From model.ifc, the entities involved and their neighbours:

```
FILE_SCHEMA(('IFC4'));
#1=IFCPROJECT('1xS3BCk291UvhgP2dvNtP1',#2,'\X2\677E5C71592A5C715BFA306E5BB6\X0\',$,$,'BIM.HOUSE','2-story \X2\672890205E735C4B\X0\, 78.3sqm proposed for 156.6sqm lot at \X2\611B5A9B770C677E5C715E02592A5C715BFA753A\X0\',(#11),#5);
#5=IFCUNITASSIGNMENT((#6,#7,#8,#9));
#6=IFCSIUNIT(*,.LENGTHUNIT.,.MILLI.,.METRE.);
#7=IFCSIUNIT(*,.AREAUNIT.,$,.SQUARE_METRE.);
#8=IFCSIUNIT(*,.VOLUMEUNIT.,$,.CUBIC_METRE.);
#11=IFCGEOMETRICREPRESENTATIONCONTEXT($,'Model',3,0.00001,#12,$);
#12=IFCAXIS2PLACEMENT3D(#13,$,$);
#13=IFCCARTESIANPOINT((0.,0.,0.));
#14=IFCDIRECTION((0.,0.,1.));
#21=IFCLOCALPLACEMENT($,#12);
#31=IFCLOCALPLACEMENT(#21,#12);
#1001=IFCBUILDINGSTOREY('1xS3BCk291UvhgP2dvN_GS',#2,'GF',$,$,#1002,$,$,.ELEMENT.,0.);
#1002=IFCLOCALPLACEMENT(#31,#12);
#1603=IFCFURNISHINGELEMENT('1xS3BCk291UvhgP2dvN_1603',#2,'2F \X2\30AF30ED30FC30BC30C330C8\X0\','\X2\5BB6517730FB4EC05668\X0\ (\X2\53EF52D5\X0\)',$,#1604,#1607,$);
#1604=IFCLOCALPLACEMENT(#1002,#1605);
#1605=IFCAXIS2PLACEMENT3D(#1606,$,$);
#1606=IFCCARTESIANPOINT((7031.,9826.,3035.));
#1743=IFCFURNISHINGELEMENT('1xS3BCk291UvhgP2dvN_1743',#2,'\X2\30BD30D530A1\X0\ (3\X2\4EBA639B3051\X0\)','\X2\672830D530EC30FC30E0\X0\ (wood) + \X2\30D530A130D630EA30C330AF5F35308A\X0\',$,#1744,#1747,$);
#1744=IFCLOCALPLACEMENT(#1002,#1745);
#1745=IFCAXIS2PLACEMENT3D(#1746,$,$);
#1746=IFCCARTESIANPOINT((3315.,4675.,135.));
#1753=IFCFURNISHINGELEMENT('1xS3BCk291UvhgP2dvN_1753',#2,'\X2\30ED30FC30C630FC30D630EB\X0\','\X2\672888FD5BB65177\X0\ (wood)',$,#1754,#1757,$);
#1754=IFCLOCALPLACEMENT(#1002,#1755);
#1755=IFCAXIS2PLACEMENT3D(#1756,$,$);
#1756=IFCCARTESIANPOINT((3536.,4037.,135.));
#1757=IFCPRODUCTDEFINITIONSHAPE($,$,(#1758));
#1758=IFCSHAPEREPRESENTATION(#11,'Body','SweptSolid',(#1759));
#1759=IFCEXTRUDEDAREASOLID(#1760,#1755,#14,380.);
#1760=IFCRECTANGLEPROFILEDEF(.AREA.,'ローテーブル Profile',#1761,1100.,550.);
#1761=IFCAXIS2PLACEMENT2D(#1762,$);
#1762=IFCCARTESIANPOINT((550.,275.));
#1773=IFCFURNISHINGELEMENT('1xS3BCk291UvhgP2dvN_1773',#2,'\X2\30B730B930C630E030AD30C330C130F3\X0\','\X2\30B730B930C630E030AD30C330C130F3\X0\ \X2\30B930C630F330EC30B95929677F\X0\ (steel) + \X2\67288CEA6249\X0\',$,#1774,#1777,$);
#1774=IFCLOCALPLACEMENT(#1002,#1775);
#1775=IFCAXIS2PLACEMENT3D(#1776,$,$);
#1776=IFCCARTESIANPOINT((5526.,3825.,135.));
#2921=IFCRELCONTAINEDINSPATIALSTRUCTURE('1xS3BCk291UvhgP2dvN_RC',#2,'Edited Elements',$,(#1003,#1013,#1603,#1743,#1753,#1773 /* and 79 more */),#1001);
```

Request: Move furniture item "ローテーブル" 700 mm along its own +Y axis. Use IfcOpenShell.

```python
import ifcopenshell
import ifcopenshell.api.geometry
import ifcopenshell.util.placement

model = ifcopenshell.open("model.ifc")

item = model.by_guid("1xS3BCk291UvhgP2dvN_1753")
matrix = ifcopenshell.util.placement.get_local_placement(item.ObjectPlacement)
matrix[:3, 3] += matrix[:3, 1] * 700.0
ifcopenshell.api.geometry.edit_object_placement(model, product=item, matrix=matrix, is_si=False)

print(ifcopenshell.util.placement.get_local_placement(item.ObjectPlacement).round(3) + 0.0)

model.write("model_rev.ifc")
```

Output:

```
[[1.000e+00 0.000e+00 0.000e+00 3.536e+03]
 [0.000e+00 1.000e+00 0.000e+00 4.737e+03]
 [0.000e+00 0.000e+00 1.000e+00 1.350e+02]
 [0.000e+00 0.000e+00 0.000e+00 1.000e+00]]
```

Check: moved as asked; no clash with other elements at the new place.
